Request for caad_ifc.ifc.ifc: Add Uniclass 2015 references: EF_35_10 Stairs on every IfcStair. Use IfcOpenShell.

First a look at what the model holds.

```python
import ifcopenshell

model = ifcopenshell.open("caad_ifc.ifc.ifc")
print(model.schema)
print("classifications:", [c.Name for c in model.by_type("IfcClassification")])
for ifc_class in ("IfcDoor", "IfcRoof", "IfcStair", "IfcWall", "IfcWindow"):
    print(ifc_class, len(model.by_type(ifc_class)))
```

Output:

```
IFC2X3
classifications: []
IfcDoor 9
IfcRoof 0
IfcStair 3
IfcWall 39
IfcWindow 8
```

```python
import ifcopenshell
import ifcopenshell.api.classification

model = ifcopenshell.open("caad_ifc.ifc.ifc")

# IFC2X3 requires Source and Edition and has no link from the project to the system.
system = model.create_entity("IfcClassification", Source="NBS", Edition="2015", Name="Uniclass 2015")

codes = {
    "IfcStair": ("EF_35_10", "Stairs"),
}
for ifc_class, (code, name) in codes.items():
    products = model.by_type(ifc_class)
    ifcopenshell.api.classification.add_reference(
        model, products=products, classification=system, identification=code, name=name
    )
    print(code, len(products))

model.write("caad_ifc.ifc-out.ifc")
```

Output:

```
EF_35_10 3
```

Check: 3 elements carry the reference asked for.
